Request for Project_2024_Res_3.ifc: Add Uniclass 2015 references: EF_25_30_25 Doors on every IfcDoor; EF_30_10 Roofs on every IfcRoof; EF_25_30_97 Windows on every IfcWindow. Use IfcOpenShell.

First a look at what the model holds.

```python
import ifcopenshell

model = ifcopenshell.open("Project_2024_Res_3.ifc")
print(model.schema)
print("classifications:", [c.Name for c in model.by_type("IfcClassification")])
for ifc_class in ("IfcDoor", "IfcRoof", "IfcStair", "IfcWall", "IfcWindow"):
    print(ifc_class, len(model.by_type(ifc_class)))
```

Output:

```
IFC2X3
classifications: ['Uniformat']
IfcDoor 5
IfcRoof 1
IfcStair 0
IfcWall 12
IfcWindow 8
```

```python
import ifcopenshell
import ifcopenshell.api.classification

model = ifcopenshell.open("Project_2024_Res_3.ifc")

# IFC2X3 requires Source and Edition and has no link from the project to the system.
system = model.create_entity("IfcClassification", Source="NBS", Edition="2015", Name="Uniclass 2015")

codes = {
    "IfcDoor": ("EF_25_30_25", "Doors"),
    "IfcRoof": ("EF_30_10", "Roofs"),
    "IfcWindow": ("EF_25_30_97", "Windows"),
}
for ifc_class, (code, name) in codes.items():
    products = model.by_type(ifc_class)
    ifcopenshell.api.classification.add_reference(
        model, products=products, classification=system, identification=code, name=name
    )
    print(code, len(products))

model.write("Project_2024_Res_3_v2.ifc")
```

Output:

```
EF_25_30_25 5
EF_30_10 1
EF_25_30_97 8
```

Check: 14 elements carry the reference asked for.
